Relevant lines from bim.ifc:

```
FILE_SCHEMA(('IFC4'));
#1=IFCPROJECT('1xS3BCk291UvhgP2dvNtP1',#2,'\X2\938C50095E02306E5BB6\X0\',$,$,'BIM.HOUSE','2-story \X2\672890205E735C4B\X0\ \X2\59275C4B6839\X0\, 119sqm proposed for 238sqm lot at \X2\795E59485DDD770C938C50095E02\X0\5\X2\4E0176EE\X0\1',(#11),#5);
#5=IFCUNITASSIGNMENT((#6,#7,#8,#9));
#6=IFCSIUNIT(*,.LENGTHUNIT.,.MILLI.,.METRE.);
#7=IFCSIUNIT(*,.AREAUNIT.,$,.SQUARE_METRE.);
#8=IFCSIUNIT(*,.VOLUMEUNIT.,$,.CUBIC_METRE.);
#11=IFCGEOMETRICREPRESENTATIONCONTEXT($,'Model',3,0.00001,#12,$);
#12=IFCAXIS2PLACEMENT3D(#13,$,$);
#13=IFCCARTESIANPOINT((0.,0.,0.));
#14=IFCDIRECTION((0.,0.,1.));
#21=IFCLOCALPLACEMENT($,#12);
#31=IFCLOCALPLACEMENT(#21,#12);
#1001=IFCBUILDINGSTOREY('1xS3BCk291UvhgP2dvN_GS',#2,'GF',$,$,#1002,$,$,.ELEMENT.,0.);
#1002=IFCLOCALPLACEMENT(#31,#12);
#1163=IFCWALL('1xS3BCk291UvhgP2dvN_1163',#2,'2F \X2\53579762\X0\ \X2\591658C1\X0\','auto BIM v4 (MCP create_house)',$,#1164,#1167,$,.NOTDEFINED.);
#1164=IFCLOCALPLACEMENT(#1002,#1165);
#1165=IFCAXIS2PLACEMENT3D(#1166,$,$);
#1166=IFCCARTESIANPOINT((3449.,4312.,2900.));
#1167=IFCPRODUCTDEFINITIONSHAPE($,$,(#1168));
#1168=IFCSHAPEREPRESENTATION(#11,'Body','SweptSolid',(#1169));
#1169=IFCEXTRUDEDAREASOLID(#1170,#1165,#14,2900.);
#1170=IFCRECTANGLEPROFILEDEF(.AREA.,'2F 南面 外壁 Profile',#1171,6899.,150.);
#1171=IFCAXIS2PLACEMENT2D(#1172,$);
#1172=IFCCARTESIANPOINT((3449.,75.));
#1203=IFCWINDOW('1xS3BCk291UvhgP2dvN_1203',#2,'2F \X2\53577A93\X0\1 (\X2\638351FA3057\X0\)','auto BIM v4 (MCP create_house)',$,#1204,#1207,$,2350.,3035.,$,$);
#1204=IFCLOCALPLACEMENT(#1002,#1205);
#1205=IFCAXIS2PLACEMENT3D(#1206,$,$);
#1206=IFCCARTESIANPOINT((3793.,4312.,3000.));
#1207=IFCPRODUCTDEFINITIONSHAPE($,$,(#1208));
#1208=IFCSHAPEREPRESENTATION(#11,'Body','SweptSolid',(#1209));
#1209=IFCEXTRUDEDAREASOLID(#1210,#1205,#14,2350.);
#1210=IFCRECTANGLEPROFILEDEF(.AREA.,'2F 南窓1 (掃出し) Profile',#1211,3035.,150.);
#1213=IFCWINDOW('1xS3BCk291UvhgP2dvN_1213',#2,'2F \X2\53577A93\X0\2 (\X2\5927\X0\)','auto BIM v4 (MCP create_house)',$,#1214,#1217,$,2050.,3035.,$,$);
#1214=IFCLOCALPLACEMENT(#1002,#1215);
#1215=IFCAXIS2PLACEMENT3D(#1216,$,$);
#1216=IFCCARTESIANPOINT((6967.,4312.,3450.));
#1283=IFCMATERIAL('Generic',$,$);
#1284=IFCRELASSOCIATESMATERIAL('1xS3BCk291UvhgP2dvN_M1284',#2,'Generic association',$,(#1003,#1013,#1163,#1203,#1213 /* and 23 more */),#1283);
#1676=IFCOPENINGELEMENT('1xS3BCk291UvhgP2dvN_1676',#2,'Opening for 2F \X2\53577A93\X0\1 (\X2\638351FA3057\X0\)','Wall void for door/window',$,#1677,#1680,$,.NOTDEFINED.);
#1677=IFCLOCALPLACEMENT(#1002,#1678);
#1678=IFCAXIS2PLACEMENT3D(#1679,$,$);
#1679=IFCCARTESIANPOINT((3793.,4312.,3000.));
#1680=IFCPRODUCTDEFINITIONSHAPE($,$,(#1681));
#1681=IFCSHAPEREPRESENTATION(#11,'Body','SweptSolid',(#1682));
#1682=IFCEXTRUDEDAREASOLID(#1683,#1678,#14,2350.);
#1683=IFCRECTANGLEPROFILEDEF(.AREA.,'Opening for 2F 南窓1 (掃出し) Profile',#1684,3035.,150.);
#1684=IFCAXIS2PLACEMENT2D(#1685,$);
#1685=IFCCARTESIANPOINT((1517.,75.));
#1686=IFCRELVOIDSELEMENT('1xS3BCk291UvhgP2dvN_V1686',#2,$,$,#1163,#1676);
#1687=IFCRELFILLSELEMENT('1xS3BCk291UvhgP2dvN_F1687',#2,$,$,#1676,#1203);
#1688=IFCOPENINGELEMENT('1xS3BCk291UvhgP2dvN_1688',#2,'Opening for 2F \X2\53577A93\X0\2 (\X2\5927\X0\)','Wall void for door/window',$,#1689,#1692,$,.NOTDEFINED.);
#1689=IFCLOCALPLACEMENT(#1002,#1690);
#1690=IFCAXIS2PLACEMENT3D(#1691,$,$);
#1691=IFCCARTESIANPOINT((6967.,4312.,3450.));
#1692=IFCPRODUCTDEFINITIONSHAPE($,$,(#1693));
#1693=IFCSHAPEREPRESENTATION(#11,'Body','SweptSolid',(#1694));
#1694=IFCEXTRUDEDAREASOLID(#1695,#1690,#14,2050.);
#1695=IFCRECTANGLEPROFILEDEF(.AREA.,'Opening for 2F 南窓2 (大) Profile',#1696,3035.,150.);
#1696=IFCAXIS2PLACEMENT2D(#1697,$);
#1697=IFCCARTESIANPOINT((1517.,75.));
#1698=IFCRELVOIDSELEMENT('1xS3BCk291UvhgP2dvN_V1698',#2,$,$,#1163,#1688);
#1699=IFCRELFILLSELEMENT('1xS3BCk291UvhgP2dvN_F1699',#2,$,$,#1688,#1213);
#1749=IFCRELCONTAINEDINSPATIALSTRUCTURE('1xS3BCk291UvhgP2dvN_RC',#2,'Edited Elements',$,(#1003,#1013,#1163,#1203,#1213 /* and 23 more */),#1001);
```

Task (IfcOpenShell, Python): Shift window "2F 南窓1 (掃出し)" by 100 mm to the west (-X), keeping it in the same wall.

```python
import ifcopenshell
import ifcopenshell.api.geometry
import ifcopenshell.util.placement
import ifcopenshell.util.unit

model = ifcopenshell.open("bim.ifc")
unit_scale = ifcopenshell.util.unit.calculate_unit_scale(model)

window = model.by_guid("1xS3BCk291UvhgP2dvN_1203")
opening = window.FillsVoids[0].RelatingOpeningElement
wall = opening.VoidsElements[0].RelatingBuildingElement

wall_matrix = ifcopenshell.util.placement.get_local_placement(wall.ObjectPlacement)
shift = wall_matrix[:3, 0] * -0.1 / unit_scale
before = ifcopenshell.util.placement.get_local_placement(window.ObjectPlacement)[:3, 3].copy()

# The window is not placed relative to its opening, so move both.
for product in (opening, window):
    matrix = ifcopenshell.util.placement.get_local_placement(product.ObjectPlacement)
    matrix[:3, 3] += shift
    ifcopenshell.api.geometry.edit_object_placement(model, product=product, matrix=matrix, is_si=False)

after = ifcopenshell.util.placement.get_local_placement(window.ObjectPlacement)[:3, 3]
print("window moved by", (after - before).round(3) + 0.0)

model.write("bim_updated.ifc")
```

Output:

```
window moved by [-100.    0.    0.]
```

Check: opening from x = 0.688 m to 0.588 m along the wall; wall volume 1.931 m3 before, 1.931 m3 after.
